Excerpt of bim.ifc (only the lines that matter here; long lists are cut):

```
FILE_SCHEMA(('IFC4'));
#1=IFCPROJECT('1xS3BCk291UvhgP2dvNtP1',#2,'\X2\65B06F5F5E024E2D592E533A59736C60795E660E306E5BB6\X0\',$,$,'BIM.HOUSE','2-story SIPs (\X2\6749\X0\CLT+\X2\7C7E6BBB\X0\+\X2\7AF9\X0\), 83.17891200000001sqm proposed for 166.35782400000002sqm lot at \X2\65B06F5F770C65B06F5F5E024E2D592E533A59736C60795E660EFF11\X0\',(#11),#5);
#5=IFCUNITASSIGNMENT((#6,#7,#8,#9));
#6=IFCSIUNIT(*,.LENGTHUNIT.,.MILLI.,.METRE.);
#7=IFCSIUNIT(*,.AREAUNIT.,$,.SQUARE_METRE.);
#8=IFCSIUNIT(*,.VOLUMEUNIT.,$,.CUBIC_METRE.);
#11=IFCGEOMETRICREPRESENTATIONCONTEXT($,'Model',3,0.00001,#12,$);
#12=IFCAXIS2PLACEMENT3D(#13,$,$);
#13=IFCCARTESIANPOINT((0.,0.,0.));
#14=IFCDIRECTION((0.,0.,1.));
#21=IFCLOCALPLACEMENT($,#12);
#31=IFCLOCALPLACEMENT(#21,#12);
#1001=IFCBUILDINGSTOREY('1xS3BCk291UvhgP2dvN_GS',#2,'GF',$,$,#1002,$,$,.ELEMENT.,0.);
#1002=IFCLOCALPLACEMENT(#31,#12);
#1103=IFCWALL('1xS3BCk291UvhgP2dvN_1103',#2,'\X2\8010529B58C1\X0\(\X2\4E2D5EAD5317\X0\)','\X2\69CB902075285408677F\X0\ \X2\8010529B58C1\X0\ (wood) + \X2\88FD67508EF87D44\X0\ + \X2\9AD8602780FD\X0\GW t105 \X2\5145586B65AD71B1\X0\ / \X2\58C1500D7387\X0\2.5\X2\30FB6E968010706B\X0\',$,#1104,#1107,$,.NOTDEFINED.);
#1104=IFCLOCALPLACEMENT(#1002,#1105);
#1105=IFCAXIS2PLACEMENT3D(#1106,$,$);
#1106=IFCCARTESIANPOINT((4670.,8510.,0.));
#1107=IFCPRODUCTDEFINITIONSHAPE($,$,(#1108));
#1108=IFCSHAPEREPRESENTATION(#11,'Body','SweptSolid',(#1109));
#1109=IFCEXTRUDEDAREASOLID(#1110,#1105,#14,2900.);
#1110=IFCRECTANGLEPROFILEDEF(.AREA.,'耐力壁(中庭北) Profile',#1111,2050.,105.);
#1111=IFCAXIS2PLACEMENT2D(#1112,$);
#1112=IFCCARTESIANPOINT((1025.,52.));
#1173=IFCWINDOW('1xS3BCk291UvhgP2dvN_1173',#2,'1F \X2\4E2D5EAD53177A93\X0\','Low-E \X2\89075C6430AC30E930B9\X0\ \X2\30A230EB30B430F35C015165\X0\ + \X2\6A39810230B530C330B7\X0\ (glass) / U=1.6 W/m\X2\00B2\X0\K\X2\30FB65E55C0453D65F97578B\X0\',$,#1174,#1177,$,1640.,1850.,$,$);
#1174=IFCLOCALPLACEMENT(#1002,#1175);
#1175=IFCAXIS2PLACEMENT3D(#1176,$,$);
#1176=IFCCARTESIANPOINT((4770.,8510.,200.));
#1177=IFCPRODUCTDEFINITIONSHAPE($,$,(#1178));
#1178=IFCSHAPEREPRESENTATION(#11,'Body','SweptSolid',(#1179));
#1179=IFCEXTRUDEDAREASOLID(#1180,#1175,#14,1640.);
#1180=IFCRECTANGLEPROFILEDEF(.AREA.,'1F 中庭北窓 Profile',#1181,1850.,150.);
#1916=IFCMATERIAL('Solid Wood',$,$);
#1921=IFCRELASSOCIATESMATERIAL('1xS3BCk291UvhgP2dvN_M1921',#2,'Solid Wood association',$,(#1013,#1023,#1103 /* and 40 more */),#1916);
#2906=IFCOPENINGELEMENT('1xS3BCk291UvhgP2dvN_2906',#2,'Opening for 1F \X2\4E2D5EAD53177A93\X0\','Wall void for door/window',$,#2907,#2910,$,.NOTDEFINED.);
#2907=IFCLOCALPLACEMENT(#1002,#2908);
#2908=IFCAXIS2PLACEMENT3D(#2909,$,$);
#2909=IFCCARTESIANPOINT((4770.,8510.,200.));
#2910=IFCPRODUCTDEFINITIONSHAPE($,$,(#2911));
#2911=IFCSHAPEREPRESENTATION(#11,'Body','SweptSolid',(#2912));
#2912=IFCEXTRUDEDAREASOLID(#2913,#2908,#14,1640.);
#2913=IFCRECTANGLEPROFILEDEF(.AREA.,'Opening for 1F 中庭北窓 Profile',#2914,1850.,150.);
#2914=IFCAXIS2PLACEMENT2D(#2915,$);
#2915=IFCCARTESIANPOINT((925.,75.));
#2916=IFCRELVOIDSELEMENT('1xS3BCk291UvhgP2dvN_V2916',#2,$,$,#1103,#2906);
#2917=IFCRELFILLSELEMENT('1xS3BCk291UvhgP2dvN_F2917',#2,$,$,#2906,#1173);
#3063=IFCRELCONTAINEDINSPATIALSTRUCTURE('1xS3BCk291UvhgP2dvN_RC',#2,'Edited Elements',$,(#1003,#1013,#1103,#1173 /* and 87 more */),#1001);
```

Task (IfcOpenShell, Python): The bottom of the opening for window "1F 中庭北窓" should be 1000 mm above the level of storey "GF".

```python
import numpy as np
import ifcopenshell
import ifcopenshell.api.geometry
import ifcopenshell.geom
import ifcopenshell.util.element
import ifcopenshell.util.placement
import ifcopenshell.util.shape
import ifcopenshell.util.unit

model = ifcopenshell.open("bim.ifc")
unit_scale = ifcopenshell.util.unit.calculate_unit_scale(model)

window = model.by_guid("1xS3BCk291UvhgP2dvN_1173")
opening = window.FillsVoids[0].RelatingOpeningElement
storey = ifcopenshell.util.element.get_container(window, ifc_class="IfcBuildingStorey")
level = ifcopenshell.util.placement.get_local_placement(storey.ObjectPlacement)[2, 3]

# The opening's origin need not be at the sill, so measure its lowest point.
shape = ifcopenshell.geom.create_shape(ifcopenshell.geom.settings(), opening)
bottom = ifcopenshell.util.shape.get_shape_bottom_elevation(shape, shape.geometry) / unit_scale
dz = level + 1000.0 - bottom

shift = np.array([0.0, 0.0, dz])
# The window is not placed relative to its opening, so move both.
for product in (opening, window):
    matrix = ifcopenshell.util.placement.get_local_placement(product.ObjectPlacement)
    matrix[:3, 3] += shift
    ifcopenshell.api.geometry.edit_object_placement(model, product=product, matrix=matrix, is_si=False)

print(f"moved by {dz * unit_scale:+.3f} m")

model.write("bim_updated.ifc")
```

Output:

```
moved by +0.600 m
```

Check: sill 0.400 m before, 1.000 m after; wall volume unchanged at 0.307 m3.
